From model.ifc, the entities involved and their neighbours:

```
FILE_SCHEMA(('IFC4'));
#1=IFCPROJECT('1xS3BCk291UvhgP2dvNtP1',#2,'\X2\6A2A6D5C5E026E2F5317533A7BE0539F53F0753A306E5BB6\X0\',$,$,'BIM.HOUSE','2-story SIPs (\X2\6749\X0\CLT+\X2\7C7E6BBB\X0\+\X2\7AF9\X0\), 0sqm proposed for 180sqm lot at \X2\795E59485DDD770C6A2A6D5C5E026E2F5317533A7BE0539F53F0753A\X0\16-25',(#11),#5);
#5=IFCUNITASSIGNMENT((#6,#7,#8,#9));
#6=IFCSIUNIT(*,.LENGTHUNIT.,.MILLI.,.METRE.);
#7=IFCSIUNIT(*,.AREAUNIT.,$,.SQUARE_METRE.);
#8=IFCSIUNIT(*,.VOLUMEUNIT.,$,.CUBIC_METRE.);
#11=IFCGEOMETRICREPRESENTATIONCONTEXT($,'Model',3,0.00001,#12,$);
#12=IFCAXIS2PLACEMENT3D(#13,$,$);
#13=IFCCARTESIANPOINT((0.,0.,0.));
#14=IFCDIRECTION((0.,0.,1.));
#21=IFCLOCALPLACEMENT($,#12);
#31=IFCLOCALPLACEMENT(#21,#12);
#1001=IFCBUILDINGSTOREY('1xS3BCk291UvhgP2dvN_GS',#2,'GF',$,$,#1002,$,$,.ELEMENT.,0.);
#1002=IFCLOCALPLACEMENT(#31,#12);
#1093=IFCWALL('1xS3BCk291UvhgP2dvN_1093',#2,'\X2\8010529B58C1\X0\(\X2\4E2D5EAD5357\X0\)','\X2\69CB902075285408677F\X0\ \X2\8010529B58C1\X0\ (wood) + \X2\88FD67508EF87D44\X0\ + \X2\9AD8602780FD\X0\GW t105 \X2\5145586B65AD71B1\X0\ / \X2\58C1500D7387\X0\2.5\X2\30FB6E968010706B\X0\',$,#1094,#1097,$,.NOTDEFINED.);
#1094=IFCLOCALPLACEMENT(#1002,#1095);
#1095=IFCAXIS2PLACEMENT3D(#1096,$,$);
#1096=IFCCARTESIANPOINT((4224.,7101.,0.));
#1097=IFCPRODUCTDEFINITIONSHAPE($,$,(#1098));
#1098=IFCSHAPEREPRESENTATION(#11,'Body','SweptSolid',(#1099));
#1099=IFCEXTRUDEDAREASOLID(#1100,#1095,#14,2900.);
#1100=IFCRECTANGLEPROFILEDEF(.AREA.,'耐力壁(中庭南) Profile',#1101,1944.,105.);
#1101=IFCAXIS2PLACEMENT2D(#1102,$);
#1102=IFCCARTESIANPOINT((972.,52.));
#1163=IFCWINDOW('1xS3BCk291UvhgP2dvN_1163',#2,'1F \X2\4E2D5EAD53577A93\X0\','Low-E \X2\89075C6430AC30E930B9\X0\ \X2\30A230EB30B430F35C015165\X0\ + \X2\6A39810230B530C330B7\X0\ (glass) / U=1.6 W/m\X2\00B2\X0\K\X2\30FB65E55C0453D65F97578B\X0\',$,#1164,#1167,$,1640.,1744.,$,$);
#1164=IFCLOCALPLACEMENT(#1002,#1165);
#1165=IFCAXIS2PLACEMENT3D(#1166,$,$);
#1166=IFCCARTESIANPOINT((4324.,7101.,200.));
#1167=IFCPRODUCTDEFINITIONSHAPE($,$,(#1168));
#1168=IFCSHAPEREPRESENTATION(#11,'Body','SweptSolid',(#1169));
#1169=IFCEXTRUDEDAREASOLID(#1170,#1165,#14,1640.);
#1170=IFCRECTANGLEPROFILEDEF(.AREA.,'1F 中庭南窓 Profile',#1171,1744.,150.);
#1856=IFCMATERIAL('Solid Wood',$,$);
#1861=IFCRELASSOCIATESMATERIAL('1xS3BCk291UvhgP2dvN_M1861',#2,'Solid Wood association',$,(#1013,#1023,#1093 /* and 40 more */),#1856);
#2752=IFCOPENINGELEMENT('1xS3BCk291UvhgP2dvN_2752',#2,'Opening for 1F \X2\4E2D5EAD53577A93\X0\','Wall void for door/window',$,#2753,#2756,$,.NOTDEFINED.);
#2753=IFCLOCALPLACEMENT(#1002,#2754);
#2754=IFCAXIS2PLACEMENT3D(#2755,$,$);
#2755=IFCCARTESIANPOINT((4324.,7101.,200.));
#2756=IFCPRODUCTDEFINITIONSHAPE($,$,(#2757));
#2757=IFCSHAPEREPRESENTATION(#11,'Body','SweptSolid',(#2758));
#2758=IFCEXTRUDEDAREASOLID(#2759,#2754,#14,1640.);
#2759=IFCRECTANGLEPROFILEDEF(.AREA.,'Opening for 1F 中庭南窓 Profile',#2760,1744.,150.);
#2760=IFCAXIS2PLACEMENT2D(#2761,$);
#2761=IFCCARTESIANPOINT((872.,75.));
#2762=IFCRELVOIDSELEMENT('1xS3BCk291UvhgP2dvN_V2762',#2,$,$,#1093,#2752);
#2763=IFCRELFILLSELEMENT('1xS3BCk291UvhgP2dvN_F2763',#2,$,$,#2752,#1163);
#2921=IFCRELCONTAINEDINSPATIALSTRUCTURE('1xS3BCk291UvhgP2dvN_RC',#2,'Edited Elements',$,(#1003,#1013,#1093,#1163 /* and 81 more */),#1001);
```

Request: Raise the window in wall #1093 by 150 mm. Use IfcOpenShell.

```python
import numpy as np
import ifcopenshell
import ifcopenshell.api.geometry
import ifcopenshell.util.placement
import ifcopenshell.util.unit

model = ifcopenshell.open("model.ifc")
unit_scale = ifcopenshell.util.unit.calculate_unit_scale(model)

window = model.by_guid("1xS3BCk291UvhgP2dvN_1163")
opening = window.FillsVoids[0].RelatingOpeningElement
dz = 150.0

shift = np.array([0.0, 0.0, dz])
# The window is not placed relative to its opening, so move both.
for product in (opening, window):
    matrix = ifcopenshell.util.placement.get_local_placement(product.ObjectPlacement)
    matrix[:3, 3] += shift
    ifcopenshell.api.geometry.edit_object_placement(model, product=product, matrix=matrix, is_si=False)

print(f"moved by {dz * unit_scale:+.3f} m")

model.write("model_v2.ifc")
```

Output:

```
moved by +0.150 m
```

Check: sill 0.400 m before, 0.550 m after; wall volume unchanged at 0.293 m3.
